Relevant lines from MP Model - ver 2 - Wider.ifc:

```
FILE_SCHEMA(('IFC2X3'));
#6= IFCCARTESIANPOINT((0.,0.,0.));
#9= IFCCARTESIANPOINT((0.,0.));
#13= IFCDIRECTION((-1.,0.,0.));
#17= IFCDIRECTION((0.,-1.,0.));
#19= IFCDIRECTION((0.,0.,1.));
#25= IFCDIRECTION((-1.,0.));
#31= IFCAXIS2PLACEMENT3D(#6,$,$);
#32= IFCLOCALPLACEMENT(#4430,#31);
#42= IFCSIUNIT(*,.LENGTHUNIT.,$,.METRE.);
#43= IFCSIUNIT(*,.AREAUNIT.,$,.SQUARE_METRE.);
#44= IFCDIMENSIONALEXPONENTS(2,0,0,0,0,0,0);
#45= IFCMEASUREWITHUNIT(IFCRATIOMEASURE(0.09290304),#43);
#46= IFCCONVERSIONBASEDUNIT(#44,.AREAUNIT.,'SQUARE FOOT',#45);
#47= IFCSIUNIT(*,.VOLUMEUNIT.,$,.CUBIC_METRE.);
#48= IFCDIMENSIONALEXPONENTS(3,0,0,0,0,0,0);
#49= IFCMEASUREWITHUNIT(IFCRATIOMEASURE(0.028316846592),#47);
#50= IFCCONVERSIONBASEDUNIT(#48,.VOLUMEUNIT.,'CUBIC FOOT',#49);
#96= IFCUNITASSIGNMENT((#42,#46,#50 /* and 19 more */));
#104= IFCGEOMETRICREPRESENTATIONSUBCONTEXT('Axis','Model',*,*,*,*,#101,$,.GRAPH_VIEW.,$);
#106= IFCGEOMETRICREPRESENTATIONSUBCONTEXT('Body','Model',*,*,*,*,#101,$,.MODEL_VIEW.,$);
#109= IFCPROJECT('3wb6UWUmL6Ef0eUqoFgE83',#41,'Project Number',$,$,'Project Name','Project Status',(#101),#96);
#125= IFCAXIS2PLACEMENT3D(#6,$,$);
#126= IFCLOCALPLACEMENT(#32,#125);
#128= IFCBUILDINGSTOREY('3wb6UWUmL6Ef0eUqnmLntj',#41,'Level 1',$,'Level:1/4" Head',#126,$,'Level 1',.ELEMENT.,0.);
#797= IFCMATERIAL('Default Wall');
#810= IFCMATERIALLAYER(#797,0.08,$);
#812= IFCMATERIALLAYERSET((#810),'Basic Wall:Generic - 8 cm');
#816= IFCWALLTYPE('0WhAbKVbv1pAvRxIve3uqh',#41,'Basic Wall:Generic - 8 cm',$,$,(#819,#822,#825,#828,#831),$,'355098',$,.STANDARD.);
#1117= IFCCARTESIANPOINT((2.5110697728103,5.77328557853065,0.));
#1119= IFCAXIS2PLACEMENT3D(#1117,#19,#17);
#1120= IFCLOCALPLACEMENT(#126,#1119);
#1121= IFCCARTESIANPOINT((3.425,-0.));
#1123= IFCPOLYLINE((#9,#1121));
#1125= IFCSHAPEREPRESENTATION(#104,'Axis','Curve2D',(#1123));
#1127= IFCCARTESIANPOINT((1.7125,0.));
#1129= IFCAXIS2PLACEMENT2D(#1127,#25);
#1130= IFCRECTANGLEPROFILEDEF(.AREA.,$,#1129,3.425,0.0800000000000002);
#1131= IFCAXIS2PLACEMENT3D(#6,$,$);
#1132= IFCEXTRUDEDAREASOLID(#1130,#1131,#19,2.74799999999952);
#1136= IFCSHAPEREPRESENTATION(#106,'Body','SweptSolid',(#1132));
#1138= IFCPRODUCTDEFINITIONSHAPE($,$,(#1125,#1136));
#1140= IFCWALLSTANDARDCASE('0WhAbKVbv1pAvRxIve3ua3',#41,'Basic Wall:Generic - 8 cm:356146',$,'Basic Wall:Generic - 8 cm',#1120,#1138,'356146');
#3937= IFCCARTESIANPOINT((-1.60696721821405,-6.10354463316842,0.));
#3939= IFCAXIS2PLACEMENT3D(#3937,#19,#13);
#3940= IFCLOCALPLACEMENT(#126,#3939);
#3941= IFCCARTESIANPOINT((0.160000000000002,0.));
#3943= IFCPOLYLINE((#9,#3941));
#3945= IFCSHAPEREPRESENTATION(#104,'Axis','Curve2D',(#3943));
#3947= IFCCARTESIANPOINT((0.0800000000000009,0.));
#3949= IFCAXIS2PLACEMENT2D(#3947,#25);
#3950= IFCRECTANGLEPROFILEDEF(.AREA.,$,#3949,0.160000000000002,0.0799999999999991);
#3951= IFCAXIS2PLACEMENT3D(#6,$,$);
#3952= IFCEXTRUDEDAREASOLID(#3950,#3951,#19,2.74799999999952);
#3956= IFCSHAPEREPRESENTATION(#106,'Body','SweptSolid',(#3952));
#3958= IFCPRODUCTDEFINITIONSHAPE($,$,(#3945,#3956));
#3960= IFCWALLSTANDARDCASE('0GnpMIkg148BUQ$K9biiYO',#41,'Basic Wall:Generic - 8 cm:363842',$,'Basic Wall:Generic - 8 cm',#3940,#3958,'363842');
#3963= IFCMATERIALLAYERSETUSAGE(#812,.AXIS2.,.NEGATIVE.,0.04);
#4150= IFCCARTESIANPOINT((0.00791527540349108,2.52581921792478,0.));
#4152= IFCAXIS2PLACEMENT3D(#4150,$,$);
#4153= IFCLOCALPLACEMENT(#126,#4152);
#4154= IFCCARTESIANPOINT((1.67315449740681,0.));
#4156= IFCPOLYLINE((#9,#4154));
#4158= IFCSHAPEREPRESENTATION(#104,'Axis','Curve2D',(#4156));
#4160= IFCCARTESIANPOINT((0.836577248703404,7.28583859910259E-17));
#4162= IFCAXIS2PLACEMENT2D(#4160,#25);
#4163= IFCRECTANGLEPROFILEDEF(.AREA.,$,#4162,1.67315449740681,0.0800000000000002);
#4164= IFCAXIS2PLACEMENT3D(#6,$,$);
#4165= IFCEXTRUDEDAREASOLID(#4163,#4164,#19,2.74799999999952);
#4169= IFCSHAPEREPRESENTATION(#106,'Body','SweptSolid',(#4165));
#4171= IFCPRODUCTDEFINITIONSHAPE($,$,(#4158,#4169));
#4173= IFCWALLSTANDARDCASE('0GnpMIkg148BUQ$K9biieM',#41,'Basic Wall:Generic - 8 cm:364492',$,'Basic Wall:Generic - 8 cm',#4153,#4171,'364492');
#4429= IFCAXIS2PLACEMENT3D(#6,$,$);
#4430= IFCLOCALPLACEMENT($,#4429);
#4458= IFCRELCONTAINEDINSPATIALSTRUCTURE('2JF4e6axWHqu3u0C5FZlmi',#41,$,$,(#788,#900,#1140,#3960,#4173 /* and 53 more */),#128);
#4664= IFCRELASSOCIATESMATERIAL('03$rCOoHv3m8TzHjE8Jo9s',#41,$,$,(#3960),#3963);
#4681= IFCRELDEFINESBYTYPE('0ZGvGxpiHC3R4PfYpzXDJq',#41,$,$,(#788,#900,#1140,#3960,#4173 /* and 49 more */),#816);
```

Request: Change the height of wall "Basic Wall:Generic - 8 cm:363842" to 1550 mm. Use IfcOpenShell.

```python
import ifcopenshell
import ifcopenshell.geom
import ifcopenshell.util.representation
import ifcopenshell.util.shape
import ifcopenshell.util.unit

model = ifcopenshell.open("MP Model - ver 2 - Wider.ifc")
unit_scale = ifcopenshell.util.unit.calculate_unit_scale(model)
settings = ifcopenshell.geom.settings()


def volume(element):
    """Net volume in cubic metres, openings subtracted."""
    shape = ifcopenshell.geom.create_shape(settings, element)
    return ifcopenshell.util.shape.get_volume(shape.geometry)


wall = model.by_guid("0GnpMIkg148BUQ$K9biiYO")
before = volume(wall)

body = ifcopenshell.util.representation.get_representation(wall, "Model", "Body")
solid = body.Items[0]
old_height = solid.Depth
solid.Depth = 1.55 / unit_scale
after = volume(wall)

print(f"height {old_height:g} -> {solid.Depth:g}, volume {before:.3f} -> {after:.3f} m3")

model.write("MP Model - ver 2 - Wider_v2.ifc")
```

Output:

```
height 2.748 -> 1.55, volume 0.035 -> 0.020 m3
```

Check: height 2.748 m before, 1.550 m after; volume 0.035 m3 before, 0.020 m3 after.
